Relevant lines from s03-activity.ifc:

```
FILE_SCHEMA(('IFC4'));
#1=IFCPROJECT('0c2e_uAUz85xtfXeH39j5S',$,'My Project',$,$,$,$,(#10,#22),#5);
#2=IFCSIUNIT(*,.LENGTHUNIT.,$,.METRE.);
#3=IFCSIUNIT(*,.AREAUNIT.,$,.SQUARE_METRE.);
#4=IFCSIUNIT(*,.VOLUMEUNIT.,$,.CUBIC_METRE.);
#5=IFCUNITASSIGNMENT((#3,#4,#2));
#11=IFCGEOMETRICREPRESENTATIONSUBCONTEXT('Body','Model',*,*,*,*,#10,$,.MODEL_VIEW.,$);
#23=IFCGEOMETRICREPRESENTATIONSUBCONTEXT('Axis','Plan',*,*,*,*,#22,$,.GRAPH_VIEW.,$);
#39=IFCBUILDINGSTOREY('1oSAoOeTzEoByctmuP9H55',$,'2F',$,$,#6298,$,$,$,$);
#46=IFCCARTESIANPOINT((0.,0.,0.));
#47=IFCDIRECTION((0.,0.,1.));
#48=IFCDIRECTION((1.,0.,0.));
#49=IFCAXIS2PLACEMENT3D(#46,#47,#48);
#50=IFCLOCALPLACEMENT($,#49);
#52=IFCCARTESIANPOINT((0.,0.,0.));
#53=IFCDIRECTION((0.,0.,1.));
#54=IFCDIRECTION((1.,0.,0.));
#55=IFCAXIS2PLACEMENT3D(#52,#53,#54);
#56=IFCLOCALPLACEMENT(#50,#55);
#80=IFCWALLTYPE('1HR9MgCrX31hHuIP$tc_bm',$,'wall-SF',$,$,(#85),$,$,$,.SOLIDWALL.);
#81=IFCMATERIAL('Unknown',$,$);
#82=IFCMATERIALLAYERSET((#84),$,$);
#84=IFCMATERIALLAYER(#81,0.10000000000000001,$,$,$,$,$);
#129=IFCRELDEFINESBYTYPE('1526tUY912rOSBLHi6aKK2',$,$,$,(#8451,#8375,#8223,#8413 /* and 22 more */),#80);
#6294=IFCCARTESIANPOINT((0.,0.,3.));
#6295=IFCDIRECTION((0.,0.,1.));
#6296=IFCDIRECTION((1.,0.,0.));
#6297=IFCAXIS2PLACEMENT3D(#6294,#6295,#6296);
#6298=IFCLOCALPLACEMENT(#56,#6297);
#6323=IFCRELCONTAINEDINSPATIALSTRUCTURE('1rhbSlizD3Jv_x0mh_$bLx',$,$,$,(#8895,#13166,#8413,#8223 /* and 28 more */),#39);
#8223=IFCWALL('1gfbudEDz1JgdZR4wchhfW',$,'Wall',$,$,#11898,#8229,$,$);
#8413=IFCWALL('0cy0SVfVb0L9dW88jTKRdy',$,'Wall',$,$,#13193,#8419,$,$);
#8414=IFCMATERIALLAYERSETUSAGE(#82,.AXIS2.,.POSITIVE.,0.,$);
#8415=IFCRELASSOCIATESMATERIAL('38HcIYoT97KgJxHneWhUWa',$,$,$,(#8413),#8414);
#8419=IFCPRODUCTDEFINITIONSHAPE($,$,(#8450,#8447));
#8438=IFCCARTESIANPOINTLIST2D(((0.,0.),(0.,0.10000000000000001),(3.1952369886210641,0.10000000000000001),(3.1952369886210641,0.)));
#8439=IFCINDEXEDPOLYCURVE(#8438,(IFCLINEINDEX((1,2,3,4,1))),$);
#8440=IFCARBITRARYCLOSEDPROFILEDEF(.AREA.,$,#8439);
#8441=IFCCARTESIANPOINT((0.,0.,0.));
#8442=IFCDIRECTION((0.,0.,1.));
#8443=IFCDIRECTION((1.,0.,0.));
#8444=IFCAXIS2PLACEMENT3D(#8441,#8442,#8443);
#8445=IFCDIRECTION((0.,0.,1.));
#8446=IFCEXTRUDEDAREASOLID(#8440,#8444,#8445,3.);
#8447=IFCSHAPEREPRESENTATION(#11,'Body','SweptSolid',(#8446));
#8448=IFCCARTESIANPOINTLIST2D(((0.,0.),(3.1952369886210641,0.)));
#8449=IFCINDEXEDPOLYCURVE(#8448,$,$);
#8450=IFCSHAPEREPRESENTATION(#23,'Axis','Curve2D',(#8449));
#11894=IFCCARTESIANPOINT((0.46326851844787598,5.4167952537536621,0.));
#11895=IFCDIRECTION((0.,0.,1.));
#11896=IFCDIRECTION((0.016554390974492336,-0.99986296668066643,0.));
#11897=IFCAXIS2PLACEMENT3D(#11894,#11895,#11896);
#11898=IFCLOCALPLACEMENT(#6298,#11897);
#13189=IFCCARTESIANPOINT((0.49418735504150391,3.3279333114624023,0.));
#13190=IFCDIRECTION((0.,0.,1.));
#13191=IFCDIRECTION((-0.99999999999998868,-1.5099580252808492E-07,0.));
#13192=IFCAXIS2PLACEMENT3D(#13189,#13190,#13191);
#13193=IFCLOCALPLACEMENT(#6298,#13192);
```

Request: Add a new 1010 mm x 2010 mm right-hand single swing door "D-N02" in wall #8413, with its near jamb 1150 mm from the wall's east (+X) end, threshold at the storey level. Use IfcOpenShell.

```python
import numpy as np
import ifcopenshell
import ifcopenshell.api.feature
import ifcopenshell.api.geometry
import ifcopenshell.api.root
import ifcopenshell.api.spatial
import ifcopenshell.geom
import ifcopenshell.util.element
import ifcopenshell.util.placement
import ifcopenshell.util.representation
import ifcopenshell.util.shape
import ifcopenshell.util.unit

model = ifcopenshell.open("s03-activity.ifc")
unit_scale = ifcopenshell.util.unit.calculate_unit_scale(model)
settings = ifcopenshell.geom.settings()


def volume(element):
    """Net volume in cubic metres, openings subtracted."""
    shape = ifcopenshell.geom.create_shape(settings, element)
    return ifcopenshell.util.shape.get_volume(shape.geometry)


wall = model.by_guid("0cy0SVfVb0L9dW88jTKRdy")
storey = ifcopenshell.util.element.get_container(wall, ifc_class="IfcBuildingStorey")
context = ifcopenshell.util.representation.get_context(model, "Model", "Body", "MODEL_VIEW")
before = volume(wall)

width, height, from_end, sill = 1.01, 2.01, 1.15, 0.0  # metres

# The wall runs along its own X axis, and the end named is its -X end.
wall_shape = ifcopenshell.geom.create_shape(settings, wall)
x, y, z = ifcopenshell.util.shape.get_vertices(wall_shape.geometry).T
start = x.min() + from_end
face, thickness = float(y.min()), float(y.max() - y.min())
wall_matrix = ifcopenshell.util.placement.get_local_placement(wall.ObjectPlacement)
level = ifcopenshell.util.placement.get_local_placement(storey.ObjectPlacement)[2, 3]


def in_wall(x, y):
    """Placement at x, y metres in the wall's axes, at sill height."""
    matrix = wall_matrix.copy()
    matrix[:, 3] = wall_matrix @ np.array([x / unit_scale, y / unit_scale, 0.0, 1.0])
    matrix[2, 3] = level + sill / unit_scale
    return matrix


# Opening: a box that overshoots both wall faces by 50 mm.
opening = ifcopenshell.api.root.create_entity(model, ifc_class="IfcOpeningElement", predefined_type="OPENING")
box = ifcopenshell.api.geometry.add_wall_representation(
    model, context=context, length=width, height=height, thickness=thickness + 0.1
)
ifcopenshell.api.geometry.assign_representation(model, product=opening, representation=box)
ifcopenshell.api.geometry.edit_object_placement(model, product=opening, matrix=in_wall(start, face - 0.05), is_si=False)
ifcopenshell.api.feature.add_feature(model, feature=opening, element=wall)

door = ifcopenshell.api.root.create_entity(model, ifc_class="IfcDoor", name="D-N02", predefined_type="DOOR")
door.OverallWidth, door.OverallHeight = width / unit_scale, height / unit_scale
door.OperationType = "SINGLE_SWING_RIGHT"
body = ifcopenshell.api.geometry.add_door_representation(
    model,
    context=context,
    overall_width=door.OverallWidth,
    overall_height=door.OverallHeight,
    operation_type="SINGLE_SWING_RIGHT",
    lining_properties={"LiningDepth": thickness / unit_scale, "ThresholdDepth": thickness / unit_scale},
)
ifcopenshell.api.geometry.assign_representation(model, product=door, representation=body)
ifcopenshell.api.spatial.assign_container(model, products=[door], relating_structure=storey)
ifcopenshell.api.feature.add_filling(model, opening=opening, element=door)

# The lining spans the wall, so the door starts at the wall face.
ifcopenshell.api.geometry.edit_object_placement(model, product=door, matrix=in_wall(start, face), is_si=False)

after = volume(wall)

print(f"wall volume {before:.3f} -> {after:.3f} m3")

model.write("s03-activity-out.ifc")
```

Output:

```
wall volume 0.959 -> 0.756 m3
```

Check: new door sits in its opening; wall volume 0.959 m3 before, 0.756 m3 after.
